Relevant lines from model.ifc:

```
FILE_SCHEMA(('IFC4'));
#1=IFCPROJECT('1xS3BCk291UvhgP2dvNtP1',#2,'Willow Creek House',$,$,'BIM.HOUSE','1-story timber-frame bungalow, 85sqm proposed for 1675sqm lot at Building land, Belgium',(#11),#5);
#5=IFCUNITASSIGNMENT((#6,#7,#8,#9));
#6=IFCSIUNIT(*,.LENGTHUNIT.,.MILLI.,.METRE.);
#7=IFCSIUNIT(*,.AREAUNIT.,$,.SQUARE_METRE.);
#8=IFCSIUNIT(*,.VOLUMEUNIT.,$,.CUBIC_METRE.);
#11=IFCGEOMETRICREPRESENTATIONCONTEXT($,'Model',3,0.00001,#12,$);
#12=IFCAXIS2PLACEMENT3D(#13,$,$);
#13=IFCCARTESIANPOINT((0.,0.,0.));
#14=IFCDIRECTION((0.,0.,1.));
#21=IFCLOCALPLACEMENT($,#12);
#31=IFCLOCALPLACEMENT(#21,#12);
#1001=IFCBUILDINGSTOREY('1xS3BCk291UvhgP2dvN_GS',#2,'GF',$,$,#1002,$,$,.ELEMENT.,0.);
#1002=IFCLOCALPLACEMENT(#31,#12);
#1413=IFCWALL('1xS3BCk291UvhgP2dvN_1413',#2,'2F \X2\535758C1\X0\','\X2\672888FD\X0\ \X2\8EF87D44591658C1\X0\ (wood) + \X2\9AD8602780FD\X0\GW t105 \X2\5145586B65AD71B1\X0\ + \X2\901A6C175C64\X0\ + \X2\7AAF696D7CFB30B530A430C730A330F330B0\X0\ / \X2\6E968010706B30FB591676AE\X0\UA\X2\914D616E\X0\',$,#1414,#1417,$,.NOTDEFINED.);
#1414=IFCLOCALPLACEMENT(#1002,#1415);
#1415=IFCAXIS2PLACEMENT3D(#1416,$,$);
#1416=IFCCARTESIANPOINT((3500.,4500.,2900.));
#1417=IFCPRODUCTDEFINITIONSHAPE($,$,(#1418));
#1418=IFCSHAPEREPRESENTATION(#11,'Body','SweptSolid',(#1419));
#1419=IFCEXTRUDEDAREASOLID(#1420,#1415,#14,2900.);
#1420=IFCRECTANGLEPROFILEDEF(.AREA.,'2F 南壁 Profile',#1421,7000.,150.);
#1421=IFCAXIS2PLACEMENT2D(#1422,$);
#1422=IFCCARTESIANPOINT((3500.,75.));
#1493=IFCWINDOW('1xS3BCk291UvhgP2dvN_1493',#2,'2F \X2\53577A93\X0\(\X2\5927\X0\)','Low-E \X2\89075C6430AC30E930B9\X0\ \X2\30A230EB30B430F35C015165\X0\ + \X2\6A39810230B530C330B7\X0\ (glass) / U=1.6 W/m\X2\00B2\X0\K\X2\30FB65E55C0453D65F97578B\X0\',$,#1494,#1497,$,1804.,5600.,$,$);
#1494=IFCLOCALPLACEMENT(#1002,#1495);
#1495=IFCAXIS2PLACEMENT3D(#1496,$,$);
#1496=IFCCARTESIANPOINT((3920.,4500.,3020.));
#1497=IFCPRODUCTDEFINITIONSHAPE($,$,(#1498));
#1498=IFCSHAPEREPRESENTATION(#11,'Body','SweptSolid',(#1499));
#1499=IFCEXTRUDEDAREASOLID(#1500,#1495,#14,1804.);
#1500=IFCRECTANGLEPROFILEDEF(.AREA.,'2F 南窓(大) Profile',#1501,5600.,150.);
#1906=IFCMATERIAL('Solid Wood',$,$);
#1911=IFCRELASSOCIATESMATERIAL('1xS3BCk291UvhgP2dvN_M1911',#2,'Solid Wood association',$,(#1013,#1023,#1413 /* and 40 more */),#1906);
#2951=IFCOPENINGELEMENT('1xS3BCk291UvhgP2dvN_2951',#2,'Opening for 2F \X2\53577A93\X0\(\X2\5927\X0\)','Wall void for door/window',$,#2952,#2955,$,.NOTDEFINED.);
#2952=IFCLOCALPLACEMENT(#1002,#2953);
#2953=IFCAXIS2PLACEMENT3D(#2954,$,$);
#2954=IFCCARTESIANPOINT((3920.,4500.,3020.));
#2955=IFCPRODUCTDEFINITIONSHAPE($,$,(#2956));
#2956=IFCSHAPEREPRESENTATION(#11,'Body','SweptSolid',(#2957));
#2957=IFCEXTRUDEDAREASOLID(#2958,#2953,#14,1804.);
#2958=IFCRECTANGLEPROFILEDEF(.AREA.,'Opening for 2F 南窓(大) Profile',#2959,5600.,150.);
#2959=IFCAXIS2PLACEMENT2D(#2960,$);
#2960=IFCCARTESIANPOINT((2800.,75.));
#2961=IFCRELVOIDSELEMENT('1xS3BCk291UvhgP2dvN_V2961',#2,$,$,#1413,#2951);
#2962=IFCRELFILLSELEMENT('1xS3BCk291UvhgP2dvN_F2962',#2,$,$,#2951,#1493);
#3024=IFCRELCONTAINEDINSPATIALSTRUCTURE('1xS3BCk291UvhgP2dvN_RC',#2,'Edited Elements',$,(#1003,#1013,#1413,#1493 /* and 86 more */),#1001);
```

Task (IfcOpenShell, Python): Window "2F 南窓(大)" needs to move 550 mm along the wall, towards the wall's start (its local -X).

```python
import ifcopenshell
import ifcopenshell.api.geometry
import ifcopenshell.util.placement

model = ifcopenshell.open("model.ifc")

window = model.by_id(1493)
opening = window.FillsVoids[0].RelatingOpeningElement
wall = opening.VoidsElements[0].RelatingBuildingElement

wall_matrix = ifcopenshell.util.placement.get_local_placement(wall.ObjectPlacement)
shift = wall_matrix[:3, 0] * -550.0
before = ifcopenshell.util.placement.get_local_placement(window.ObjectPlacement)[:3, 3].copy()

# The window is not placed relative to its opening, so move both.
for product in (opening, window):
    matrix = ifcopenshell.util.placement.get_local_placement(product.ObjectPlacement)
    matrix[:3, 3] += shift
    ifcopenshell.api.geometry.edit_object_placement(model, product=product, matrix=matrix, is_si=False)

after = ifcopenshell.util.placement.get_local_placement(window.ObjectPlacement)[:3, 3]
print("window moved by", (after - before).round(3) + 0.0)

model.write("model-out.ifc")
```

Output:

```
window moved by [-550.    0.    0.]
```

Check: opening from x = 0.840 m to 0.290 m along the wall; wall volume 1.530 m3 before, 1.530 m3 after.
